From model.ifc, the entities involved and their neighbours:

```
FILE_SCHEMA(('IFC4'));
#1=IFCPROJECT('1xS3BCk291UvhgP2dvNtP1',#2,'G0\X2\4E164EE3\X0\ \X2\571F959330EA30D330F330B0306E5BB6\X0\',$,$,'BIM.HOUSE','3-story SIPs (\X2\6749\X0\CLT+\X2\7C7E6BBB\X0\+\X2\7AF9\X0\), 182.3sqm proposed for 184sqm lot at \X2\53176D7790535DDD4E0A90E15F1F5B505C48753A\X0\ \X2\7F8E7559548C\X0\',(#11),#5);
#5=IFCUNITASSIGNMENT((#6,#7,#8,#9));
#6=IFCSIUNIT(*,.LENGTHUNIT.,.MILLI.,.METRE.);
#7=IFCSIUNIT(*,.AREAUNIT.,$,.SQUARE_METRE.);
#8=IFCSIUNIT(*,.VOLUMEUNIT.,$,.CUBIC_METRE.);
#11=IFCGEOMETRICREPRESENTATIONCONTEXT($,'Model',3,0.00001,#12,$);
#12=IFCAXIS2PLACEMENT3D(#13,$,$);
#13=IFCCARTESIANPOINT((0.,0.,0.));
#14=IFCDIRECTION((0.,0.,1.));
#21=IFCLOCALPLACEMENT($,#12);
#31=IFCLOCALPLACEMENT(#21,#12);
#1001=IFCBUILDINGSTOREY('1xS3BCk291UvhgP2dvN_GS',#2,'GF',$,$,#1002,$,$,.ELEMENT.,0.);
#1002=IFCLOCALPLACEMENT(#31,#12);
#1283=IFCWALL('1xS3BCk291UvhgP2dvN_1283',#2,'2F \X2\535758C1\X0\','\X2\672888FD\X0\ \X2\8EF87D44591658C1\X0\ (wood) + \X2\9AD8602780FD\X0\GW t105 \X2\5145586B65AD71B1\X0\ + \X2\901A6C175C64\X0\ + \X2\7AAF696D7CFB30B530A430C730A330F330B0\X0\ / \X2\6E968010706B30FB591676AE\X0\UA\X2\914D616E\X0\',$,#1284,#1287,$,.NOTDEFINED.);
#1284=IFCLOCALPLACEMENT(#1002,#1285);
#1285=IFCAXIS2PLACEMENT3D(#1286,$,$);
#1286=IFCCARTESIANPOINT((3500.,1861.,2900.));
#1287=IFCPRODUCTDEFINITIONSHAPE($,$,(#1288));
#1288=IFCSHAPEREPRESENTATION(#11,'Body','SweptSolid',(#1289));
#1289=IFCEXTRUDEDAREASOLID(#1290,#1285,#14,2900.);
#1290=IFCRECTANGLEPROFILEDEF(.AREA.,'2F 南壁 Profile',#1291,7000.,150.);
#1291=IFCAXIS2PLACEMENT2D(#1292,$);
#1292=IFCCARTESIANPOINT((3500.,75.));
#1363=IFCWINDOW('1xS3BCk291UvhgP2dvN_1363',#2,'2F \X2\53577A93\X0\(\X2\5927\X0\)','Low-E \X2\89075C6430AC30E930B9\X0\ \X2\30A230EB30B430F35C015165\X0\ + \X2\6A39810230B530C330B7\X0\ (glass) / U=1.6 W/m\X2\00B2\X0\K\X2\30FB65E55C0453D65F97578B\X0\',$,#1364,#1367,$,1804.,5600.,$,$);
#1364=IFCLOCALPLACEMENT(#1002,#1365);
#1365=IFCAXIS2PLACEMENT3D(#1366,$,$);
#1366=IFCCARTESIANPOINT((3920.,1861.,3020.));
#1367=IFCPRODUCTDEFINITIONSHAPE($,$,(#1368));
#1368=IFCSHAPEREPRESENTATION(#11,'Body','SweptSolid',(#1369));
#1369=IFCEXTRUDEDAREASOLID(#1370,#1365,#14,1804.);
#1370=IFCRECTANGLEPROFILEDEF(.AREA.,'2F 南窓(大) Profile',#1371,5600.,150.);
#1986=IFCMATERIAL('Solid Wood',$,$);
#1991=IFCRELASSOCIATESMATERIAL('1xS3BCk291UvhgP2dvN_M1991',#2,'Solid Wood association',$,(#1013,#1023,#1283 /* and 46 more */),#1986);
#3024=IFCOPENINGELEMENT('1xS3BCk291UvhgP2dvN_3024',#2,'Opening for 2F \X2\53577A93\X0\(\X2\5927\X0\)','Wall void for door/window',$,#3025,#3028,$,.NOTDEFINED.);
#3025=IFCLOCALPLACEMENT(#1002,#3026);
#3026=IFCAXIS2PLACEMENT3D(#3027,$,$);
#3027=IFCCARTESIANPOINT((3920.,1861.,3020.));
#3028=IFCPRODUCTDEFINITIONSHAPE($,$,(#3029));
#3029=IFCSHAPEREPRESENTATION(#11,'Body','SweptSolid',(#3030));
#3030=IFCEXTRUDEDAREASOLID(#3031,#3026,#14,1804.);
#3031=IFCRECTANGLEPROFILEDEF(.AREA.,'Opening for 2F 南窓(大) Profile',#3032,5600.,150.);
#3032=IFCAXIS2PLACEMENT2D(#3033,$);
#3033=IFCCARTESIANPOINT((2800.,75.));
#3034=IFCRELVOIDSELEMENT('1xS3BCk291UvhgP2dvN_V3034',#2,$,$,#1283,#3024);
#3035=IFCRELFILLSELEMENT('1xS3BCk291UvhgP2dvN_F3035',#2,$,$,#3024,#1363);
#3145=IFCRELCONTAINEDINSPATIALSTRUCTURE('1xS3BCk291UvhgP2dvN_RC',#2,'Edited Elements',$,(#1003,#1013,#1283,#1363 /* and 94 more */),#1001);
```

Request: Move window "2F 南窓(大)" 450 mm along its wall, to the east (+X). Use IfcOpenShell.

```python
import ifcopenshell
import ifcopenshell.api.geometry
import ifcopenshell.util.placement
import ifcopenshell.util.unit

model = ifcopenshell.open("model.ifc")
unit_scale = ifcopenshell.util.unit.calculate_unit_scale(model)

window = model.by_guid("1xS3BCk291UvhgP2dvN_1363")
opening = window.FillsVoids[0].RelatingOpeningElement
wall = opening.VoidsElements[0].RelatingBuildingElement

wall_matrix = ifcopenshell.util.placement.get_local_placement(wall.ObjectPlacement)
shift = wall_matrix[:3, 0] * 0.45 / unit_scale
before = ifcopenshell.util.placement.get_local_placement(window.ObjectPlacement)[:3, 3].copy()

# The window is not placed relative to its opening, so move both.
for product in (opening, window):
    matrix = ifcopenshell.util.placement.get_local_placement(product.ObjectPlacement)
    matrix[:3, 3] += shift
    ifcopenshell.api.geometry.edit_object_placement(model, product=product, matrix=matrix, is_si=False)

after = ifcopenshell.util.placement.get_local_placement(window.ObjectPlacement)[:3, 3]
print("window moved by", (after - before).round(3) + 0.0)

model.write("model_edited.ifc")
```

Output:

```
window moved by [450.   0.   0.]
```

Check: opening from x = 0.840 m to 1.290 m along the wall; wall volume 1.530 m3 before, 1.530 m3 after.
